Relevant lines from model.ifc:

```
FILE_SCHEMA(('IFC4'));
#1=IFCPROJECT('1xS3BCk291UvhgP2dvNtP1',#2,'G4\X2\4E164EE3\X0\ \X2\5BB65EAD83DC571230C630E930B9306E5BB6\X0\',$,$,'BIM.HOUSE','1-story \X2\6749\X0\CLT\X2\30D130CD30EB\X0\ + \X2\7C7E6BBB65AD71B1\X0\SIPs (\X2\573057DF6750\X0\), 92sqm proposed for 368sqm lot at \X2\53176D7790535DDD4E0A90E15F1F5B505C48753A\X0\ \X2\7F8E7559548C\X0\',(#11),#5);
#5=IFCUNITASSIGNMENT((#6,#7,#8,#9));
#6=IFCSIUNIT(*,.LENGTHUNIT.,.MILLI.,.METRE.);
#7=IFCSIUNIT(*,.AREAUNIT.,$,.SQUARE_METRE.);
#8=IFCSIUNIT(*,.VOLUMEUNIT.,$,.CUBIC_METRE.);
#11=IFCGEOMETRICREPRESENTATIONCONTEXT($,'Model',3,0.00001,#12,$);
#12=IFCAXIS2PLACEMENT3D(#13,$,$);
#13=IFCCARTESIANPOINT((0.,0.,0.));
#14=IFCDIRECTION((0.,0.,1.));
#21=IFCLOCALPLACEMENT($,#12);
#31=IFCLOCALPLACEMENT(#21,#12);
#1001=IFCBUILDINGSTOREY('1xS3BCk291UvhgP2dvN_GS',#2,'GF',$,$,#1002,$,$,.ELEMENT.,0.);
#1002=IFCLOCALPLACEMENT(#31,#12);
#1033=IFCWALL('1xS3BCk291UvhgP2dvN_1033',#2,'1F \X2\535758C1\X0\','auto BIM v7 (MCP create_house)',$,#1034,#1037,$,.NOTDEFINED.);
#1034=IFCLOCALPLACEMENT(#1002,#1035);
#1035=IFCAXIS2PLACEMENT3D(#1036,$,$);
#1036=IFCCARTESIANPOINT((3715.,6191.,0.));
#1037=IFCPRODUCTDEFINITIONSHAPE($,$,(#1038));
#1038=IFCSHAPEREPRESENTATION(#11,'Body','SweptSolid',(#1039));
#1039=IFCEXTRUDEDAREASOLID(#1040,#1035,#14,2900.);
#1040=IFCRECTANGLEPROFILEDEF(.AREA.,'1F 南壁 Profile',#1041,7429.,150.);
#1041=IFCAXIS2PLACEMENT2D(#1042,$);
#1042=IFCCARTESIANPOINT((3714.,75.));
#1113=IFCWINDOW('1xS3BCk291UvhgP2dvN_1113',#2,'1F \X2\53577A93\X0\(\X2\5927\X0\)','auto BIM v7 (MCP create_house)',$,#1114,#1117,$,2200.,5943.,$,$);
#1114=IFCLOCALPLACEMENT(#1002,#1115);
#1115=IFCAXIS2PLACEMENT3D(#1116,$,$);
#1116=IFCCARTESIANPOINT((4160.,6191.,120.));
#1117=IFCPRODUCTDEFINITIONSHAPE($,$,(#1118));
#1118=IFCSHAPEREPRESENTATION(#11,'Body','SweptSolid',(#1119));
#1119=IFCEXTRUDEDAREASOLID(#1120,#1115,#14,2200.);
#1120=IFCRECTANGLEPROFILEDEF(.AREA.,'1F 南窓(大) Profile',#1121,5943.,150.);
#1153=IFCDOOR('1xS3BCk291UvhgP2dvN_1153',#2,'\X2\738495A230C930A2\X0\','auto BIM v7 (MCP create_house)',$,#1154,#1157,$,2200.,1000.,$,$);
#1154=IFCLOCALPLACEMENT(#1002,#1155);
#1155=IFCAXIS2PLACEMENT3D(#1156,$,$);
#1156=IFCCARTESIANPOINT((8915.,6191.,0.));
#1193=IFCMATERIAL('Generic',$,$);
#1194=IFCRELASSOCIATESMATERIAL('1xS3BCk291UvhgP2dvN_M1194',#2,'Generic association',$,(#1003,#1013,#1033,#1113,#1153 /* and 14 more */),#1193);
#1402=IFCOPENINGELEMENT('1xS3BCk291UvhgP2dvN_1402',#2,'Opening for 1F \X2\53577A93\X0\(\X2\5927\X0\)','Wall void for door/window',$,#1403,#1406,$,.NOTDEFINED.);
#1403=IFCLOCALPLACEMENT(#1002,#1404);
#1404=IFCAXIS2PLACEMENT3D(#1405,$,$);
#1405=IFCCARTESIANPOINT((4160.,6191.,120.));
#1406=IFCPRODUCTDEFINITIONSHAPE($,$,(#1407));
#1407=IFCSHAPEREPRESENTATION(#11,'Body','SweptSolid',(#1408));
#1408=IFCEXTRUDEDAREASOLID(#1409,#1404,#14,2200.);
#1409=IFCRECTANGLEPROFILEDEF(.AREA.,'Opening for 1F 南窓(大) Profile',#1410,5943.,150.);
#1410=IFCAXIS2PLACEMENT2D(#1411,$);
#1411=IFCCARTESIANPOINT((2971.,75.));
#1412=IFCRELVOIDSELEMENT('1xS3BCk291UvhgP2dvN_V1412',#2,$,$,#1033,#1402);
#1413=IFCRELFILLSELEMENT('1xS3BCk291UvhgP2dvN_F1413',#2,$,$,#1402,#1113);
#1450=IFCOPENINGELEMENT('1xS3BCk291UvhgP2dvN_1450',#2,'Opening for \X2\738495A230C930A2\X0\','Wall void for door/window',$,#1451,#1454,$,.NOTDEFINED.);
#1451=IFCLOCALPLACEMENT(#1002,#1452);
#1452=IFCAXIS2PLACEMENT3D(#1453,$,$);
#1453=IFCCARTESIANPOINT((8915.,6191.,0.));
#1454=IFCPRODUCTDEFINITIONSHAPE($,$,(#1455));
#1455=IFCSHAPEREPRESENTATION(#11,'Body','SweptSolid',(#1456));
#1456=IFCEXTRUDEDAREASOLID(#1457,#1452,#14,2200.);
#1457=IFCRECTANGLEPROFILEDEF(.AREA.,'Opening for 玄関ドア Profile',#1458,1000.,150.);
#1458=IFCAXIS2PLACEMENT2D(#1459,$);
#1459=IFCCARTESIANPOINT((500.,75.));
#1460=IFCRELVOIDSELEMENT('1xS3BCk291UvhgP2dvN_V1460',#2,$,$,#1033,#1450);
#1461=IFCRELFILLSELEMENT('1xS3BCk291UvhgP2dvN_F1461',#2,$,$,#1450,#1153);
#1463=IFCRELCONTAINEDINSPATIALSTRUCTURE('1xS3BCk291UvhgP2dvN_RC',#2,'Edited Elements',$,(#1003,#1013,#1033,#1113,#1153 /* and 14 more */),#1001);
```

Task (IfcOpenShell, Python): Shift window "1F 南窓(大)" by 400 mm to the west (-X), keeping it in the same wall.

```python
import ifcopenshell
import ifcopenshell.api.geometry
import ifcopenshell.util.placement

model = ifcopenshell.open("model.ifc")

window = model.by_id(1113)
opening = window.FillsVoids[0].RelatingOpeningElement
wall = opening.VoidsElements[0].RelatingBuildingElement

wall_matrix = ifcopenshell.util.placement.get_local_placement(wall.ObjectPlacement)
shift = wall_matrix[:3, 0] * -400.0
before = ifcopenshell.util.placement.get_local_placement(window.ObjectPlacement)[:3, 3].copy()

# The window is not placed relative to its opening, so move both.
for product in (opening, window):
    matrix = ifcopenshell.util.placement.get_local_placement(product.ObjectPlacement)
    matrix[:3, 3] += shift
    ifcopenshell.api.geometry.edit_object_placement(model, product=product, matrix=matrix, is_si=False)

after = ifcopenshell.util.placement.get_local_placement(window.ObjectPlacement)[:3, 3]
print("window moved by", (after - before).round(3) + 0.0)

model.write("model_edited.ifc")
```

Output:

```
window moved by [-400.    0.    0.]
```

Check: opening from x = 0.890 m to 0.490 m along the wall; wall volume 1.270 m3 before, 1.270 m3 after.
